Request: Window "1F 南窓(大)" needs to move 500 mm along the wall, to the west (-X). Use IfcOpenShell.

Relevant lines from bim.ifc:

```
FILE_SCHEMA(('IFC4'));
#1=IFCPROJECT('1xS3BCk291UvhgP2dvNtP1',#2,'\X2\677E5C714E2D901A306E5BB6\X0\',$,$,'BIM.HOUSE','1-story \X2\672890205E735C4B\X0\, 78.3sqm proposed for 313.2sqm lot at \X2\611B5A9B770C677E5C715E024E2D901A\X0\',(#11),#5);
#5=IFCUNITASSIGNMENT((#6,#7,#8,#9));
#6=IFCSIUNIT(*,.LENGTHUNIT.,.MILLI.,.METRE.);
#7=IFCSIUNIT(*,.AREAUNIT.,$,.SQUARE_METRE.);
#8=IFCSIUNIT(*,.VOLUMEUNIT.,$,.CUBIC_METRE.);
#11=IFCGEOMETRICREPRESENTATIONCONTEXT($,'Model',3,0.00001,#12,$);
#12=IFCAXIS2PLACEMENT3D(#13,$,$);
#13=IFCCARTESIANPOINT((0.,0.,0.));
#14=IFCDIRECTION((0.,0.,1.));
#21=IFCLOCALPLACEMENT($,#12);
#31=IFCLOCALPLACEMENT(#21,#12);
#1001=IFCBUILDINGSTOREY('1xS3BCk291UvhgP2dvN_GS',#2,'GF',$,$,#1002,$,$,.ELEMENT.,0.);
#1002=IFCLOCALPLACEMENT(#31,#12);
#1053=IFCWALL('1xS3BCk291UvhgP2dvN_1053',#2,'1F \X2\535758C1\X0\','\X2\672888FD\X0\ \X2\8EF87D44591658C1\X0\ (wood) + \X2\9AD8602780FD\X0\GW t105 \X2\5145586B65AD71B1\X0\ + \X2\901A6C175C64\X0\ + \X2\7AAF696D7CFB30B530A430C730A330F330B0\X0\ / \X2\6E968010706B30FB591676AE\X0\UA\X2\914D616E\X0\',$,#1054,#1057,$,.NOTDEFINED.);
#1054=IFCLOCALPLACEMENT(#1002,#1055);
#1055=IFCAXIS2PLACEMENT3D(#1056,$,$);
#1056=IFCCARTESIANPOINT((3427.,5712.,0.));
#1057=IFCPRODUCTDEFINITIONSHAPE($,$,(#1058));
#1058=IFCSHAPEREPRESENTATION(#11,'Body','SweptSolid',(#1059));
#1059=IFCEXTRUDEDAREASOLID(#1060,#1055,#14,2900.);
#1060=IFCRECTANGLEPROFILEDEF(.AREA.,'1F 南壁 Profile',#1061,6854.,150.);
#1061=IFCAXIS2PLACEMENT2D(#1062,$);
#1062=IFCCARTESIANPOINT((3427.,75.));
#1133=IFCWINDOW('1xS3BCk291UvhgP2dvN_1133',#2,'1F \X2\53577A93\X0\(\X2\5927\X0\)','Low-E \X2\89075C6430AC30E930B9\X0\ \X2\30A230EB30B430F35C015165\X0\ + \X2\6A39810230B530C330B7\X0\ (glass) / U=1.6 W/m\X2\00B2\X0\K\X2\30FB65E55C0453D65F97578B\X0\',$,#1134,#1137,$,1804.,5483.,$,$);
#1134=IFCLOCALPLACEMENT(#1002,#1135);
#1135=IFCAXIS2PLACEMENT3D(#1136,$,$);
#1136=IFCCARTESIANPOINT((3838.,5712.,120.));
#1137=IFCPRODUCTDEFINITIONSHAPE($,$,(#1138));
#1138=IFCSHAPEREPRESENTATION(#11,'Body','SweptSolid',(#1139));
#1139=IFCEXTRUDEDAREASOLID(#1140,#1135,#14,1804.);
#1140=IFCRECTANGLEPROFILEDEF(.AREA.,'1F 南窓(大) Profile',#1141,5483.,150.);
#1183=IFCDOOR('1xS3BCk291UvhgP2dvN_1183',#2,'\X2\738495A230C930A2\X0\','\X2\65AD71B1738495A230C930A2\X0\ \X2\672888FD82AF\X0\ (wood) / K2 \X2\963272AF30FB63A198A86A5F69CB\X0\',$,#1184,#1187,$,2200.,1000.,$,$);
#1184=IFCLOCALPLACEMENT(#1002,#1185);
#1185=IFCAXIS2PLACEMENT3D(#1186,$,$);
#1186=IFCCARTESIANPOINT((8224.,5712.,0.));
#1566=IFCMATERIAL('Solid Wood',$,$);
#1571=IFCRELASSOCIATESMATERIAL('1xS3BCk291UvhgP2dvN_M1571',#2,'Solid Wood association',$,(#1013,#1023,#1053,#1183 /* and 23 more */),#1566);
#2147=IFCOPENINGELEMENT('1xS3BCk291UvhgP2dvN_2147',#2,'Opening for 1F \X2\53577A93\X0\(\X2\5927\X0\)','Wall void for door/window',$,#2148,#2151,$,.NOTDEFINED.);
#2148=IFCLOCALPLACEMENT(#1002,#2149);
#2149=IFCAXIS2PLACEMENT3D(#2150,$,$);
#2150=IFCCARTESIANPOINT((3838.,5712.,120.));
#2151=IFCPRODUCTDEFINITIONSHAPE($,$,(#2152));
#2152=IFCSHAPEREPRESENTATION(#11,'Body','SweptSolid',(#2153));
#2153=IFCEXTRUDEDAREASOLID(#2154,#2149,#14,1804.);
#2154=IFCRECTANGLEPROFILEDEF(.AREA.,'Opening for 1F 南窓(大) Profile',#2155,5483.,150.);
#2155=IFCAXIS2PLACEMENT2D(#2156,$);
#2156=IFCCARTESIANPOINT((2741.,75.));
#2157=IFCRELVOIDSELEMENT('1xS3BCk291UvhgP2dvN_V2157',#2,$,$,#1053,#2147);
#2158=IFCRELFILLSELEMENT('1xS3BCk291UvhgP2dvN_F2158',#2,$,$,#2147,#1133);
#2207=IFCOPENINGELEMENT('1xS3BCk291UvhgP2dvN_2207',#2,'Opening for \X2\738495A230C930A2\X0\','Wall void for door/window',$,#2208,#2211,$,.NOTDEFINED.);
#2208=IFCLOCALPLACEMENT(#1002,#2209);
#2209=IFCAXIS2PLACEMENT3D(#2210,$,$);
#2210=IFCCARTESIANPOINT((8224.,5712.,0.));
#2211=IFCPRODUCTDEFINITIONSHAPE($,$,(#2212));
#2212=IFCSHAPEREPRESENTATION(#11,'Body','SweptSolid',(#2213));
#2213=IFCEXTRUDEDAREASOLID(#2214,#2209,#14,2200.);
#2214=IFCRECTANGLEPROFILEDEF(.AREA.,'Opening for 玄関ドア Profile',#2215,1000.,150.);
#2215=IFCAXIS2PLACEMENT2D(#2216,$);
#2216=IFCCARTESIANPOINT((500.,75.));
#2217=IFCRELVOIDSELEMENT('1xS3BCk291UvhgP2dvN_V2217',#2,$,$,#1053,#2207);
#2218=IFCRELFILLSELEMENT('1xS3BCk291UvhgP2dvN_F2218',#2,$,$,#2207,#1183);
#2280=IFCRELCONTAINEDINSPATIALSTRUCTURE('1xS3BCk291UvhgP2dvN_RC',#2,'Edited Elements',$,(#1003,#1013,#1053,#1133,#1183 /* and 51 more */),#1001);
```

```python
import ifcopenshell
import ifcopenshell.api.geometry
import ifcopenshell.util.placement
import ifcopenshell.util.unit

model = ifcopenshell.open("bim.ifc")
unit_scale = ifcopenshell.util.unit.calculate_unit_scale(model)

window = model.by_guid("1xS3BCk291UvhgP2dvN_1133")
opening = window.FillsVoids[0].RelatingOpeningElement
wall = opening.VoidsElements[0].RelatingBuildingElement

wall_matrix = ifcopenshell.util.placement.get_local_placement(wall.ObjectPlacement)
shift = wall_matrix[:3, 0] * -0.5 / unit_scale
before = ifcopenshell.util.placement.get_local_placement(window.ObjectPlacement)[:3, 3].copy()

# The window is not placed relative to its opening, so move both.
for product in (opening, window):
    matrix = ifcopenshell.util.placement.get_local_placement(product.ObjectPlacement)
    matrix[:3, 3] += shift
    ifcopenshell.api.geometry.edit_object_placement(model, product=product, matrix=matrix, is_si=False)

after = ifcopenshell.util.placement.get_local_placement(window.ObjectPlacement)[:3, 3]
print("window moved by", (after - before).round(3) + 0.0)

model.write("bim-out.ifc")
```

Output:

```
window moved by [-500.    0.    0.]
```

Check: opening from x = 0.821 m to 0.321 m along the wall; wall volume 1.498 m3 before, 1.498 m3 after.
